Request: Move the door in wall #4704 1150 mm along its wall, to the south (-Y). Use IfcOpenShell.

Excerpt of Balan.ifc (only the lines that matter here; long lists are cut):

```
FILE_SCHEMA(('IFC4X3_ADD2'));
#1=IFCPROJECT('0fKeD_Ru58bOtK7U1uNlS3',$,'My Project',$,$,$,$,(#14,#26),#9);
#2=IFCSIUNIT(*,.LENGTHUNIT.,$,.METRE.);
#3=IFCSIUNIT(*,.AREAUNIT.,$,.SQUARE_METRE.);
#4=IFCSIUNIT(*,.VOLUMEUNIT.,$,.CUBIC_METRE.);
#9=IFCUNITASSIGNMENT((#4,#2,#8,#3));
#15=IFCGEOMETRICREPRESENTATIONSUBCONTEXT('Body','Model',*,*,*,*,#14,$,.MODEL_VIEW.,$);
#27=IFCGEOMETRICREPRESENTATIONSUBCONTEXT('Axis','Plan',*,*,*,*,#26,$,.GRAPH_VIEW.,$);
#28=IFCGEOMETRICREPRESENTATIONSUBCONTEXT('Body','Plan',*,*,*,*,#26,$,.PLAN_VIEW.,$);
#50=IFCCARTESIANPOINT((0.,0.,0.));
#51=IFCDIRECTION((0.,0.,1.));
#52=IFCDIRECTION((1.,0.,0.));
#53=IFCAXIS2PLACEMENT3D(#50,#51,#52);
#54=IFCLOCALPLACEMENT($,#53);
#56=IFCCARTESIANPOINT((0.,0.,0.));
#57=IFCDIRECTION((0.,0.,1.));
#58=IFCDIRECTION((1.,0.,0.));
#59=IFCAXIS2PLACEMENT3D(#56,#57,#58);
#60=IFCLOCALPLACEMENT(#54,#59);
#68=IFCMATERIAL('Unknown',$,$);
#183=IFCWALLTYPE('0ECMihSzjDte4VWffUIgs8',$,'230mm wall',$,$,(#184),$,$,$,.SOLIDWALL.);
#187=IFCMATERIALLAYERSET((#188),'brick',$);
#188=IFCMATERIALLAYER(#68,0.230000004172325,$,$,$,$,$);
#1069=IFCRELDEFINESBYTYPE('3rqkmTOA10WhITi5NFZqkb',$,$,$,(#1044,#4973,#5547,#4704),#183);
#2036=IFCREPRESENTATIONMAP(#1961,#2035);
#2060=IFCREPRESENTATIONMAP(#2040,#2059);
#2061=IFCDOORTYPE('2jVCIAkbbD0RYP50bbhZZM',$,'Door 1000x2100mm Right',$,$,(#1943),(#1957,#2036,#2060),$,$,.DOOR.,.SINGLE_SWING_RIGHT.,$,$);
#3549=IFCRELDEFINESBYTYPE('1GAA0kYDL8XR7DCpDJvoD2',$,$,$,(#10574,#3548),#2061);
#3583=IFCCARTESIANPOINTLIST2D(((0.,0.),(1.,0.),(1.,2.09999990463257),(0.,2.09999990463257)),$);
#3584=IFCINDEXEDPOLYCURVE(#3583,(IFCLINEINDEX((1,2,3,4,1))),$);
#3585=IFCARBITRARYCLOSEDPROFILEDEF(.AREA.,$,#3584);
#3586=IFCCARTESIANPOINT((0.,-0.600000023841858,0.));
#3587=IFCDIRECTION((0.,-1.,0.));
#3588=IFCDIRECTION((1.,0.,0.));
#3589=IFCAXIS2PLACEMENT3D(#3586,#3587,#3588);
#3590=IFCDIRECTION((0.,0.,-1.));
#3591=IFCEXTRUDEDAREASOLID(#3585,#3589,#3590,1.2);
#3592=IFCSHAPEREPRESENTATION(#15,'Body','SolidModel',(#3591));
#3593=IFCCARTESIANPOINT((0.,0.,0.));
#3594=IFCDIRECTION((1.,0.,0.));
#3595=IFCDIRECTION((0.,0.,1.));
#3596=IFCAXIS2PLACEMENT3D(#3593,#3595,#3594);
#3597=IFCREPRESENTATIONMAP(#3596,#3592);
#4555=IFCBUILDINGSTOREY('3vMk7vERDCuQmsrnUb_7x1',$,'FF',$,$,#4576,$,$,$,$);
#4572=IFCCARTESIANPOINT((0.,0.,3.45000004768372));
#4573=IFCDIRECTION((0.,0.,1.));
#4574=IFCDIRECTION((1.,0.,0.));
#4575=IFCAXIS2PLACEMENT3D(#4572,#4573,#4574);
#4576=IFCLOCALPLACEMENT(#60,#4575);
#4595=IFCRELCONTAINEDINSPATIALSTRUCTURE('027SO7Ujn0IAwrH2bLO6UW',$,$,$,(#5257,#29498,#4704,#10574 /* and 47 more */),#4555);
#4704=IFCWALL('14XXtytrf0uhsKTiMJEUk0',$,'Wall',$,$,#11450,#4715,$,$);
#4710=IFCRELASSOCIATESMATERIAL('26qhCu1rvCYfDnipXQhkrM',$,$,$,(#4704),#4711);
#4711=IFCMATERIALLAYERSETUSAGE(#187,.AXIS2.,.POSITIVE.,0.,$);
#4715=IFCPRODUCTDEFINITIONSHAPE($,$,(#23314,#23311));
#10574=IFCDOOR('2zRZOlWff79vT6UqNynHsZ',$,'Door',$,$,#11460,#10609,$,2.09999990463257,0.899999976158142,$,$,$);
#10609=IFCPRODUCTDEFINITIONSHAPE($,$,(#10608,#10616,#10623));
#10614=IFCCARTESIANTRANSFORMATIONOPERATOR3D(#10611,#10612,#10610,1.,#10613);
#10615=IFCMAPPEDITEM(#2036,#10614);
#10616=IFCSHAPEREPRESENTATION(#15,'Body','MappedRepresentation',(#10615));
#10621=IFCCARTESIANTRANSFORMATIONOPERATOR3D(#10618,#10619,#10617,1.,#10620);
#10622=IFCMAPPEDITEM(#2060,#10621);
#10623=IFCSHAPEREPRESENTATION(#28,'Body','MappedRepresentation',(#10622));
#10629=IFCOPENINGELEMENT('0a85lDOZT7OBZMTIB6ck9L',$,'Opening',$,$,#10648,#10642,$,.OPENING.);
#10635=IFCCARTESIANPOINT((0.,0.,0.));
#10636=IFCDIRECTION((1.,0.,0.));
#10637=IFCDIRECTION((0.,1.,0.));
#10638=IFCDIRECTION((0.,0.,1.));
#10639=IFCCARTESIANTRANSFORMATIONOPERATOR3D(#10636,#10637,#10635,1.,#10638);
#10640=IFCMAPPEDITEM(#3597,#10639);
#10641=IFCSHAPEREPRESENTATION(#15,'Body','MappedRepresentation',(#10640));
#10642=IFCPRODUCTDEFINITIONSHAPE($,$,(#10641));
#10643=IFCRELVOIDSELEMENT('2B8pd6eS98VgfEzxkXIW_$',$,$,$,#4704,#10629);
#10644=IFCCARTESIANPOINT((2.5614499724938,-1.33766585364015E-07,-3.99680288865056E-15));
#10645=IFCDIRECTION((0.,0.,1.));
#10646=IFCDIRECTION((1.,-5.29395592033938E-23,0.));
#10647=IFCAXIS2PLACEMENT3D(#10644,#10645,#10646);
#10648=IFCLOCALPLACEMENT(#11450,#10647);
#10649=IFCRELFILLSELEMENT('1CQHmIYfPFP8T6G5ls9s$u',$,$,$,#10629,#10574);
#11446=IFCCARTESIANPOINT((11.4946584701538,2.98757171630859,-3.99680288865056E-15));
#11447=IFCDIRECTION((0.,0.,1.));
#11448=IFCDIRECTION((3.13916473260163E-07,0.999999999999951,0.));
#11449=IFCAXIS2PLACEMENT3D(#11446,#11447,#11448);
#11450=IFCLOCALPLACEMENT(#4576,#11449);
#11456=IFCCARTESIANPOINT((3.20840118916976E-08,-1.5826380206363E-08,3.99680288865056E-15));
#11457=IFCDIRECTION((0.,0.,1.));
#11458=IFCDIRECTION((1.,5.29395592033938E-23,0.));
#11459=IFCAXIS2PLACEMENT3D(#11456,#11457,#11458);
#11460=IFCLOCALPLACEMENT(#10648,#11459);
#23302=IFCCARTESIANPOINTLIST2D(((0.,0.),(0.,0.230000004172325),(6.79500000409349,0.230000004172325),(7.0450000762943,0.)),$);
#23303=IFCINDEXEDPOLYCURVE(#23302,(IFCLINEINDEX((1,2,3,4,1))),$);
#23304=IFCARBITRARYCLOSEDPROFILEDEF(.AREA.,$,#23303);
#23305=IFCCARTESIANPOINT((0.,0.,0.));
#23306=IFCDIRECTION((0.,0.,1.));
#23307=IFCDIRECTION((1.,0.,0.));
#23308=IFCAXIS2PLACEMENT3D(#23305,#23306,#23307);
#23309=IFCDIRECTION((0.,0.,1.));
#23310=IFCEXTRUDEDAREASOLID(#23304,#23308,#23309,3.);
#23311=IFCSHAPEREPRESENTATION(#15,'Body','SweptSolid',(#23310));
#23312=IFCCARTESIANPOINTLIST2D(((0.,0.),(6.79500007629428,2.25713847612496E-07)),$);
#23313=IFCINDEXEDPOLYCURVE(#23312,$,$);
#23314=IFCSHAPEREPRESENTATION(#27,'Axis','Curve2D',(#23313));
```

```python
import ifcopenshell
import ifcopenshell.api.geometry
import ifcopenshell.util.placement

model = ifcopenshell.open("Balan.ifc")

door = model.by_id(10574)
opening = door.FillsVoids[0].RelatingOpeningElement
wall = opening.VoidsElements[0].RelatingBuildingElement

wall_matrix = ifcopenshell.util.placement.get_local_placement(wall.ObjectPlacement)
shift = wall_matrix[:3, 0] * -1.15
before = ifcopenshell.util.placement.get_local_placement(door.ObjectPlacement)[:3, 3].copy()

# The door is placed relative to its opening, so it follows when the opening moves.
matrix = ifcopenshell.util.placement.get_local_placement(opening.ObjectPlacement)
matrix[:3, 3] += shift
ifcopenshell.api.geometry.edit_object_placement(
    model, product=opening, matrix=matrix, is_si=False, should_transform_children=True
)

after = ifcopenshell.util.placement.get_local_placement(door.ObjectPlacement)[:3, 3]
print("door moved by", (after - before).round(3) + 0.0)

model.write("Balan_edited.ifc")
```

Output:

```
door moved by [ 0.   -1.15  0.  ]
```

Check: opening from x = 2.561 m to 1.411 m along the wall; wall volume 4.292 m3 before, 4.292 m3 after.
